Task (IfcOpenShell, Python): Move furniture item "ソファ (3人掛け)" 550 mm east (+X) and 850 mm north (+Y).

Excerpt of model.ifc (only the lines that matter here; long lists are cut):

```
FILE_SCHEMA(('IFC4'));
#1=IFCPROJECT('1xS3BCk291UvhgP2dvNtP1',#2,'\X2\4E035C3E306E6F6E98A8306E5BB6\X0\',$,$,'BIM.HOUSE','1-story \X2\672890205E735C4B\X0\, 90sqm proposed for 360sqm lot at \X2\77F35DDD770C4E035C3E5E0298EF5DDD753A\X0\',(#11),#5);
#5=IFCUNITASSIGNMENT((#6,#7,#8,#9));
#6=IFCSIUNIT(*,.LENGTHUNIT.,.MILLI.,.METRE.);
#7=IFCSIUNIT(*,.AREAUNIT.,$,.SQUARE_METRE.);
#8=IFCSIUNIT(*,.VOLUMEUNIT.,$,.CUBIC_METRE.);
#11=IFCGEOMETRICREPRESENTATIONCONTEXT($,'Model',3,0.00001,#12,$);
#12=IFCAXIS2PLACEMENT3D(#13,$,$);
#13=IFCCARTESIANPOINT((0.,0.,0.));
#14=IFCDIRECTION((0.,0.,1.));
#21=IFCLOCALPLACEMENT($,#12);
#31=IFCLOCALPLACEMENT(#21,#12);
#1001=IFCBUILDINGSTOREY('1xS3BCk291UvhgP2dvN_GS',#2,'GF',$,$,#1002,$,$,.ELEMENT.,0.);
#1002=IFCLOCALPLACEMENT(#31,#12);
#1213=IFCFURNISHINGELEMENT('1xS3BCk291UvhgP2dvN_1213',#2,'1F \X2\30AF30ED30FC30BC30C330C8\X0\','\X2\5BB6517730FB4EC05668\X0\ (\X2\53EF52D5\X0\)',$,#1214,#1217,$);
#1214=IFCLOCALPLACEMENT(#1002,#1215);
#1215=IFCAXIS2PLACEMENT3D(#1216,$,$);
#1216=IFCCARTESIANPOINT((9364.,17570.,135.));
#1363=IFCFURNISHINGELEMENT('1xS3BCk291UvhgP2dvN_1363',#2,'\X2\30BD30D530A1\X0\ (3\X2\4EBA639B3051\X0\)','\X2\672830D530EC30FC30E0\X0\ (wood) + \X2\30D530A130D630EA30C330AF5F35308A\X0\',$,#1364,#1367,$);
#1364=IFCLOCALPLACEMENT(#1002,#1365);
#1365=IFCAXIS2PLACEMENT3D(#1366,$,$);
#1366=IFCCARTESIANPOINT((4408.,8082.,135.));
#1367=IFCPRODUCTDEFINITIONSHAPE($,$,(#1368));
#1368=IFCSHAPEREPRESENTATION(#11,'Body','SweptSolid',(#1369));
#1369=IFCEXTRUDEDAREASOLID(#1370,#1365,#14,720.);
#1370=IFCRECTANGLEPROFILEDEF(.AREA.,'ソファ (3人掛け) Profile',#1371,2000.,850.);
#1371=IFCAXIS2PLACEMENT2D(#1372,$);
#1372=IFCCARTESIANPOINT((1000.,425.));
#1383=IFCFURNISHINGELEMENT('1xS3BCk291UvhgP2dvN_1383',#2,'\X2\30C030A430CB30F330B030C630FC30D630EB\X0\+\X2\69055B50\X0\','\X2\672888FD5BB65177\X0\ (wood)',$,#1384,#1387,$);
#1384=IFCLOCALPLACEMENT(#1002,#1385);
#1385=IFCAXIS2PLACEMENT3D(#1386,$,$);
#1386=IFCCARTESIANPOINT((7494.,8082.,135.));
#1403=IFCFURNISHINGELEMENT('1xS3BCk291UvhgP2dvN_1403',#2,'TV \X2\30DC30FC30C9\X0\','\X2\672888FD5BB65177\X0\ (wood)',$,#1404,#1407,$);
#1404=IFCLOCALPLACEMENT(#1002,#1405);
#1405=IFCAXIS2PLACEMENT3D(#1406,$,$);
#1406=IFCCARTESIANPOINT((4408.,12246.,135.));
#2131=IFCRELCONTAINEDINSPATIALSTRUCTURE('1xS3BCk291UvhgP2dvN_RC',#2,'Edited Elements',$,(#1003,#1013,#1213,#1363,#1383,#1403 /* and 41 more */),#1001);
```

```python
import ifcopenshell
import ifcopenshell.api.geometry
import ifcopenshell.util.placement

model = ifcopenshell.open("model.ifc")

item = model.by_guid("1xS3BCk291UvhgP2dvN_1363")
matrix = ifcopenshell.util.placement.get_local_placement(item.ObjectPlacement)
matrix[0, 3] += 550.0
matrix[1, 3] += 850.0
ifcopenshell.api.geometry.edit_object_placement(model, product=item, matrix=matrix, is_si=False)

print(ifcopenshell.util.placement.get_local_placement(item.ObjectPlacement).round(3) + 0.0)

model.write("model_edited.ifc")
```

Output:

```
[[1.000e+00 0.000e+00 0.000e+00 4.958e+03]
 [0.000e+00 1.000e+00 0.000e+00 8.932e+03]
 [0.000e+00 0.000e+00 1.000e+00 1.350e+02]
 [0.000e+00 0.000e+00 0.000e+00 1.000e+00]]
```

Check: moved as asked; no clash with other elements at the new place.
